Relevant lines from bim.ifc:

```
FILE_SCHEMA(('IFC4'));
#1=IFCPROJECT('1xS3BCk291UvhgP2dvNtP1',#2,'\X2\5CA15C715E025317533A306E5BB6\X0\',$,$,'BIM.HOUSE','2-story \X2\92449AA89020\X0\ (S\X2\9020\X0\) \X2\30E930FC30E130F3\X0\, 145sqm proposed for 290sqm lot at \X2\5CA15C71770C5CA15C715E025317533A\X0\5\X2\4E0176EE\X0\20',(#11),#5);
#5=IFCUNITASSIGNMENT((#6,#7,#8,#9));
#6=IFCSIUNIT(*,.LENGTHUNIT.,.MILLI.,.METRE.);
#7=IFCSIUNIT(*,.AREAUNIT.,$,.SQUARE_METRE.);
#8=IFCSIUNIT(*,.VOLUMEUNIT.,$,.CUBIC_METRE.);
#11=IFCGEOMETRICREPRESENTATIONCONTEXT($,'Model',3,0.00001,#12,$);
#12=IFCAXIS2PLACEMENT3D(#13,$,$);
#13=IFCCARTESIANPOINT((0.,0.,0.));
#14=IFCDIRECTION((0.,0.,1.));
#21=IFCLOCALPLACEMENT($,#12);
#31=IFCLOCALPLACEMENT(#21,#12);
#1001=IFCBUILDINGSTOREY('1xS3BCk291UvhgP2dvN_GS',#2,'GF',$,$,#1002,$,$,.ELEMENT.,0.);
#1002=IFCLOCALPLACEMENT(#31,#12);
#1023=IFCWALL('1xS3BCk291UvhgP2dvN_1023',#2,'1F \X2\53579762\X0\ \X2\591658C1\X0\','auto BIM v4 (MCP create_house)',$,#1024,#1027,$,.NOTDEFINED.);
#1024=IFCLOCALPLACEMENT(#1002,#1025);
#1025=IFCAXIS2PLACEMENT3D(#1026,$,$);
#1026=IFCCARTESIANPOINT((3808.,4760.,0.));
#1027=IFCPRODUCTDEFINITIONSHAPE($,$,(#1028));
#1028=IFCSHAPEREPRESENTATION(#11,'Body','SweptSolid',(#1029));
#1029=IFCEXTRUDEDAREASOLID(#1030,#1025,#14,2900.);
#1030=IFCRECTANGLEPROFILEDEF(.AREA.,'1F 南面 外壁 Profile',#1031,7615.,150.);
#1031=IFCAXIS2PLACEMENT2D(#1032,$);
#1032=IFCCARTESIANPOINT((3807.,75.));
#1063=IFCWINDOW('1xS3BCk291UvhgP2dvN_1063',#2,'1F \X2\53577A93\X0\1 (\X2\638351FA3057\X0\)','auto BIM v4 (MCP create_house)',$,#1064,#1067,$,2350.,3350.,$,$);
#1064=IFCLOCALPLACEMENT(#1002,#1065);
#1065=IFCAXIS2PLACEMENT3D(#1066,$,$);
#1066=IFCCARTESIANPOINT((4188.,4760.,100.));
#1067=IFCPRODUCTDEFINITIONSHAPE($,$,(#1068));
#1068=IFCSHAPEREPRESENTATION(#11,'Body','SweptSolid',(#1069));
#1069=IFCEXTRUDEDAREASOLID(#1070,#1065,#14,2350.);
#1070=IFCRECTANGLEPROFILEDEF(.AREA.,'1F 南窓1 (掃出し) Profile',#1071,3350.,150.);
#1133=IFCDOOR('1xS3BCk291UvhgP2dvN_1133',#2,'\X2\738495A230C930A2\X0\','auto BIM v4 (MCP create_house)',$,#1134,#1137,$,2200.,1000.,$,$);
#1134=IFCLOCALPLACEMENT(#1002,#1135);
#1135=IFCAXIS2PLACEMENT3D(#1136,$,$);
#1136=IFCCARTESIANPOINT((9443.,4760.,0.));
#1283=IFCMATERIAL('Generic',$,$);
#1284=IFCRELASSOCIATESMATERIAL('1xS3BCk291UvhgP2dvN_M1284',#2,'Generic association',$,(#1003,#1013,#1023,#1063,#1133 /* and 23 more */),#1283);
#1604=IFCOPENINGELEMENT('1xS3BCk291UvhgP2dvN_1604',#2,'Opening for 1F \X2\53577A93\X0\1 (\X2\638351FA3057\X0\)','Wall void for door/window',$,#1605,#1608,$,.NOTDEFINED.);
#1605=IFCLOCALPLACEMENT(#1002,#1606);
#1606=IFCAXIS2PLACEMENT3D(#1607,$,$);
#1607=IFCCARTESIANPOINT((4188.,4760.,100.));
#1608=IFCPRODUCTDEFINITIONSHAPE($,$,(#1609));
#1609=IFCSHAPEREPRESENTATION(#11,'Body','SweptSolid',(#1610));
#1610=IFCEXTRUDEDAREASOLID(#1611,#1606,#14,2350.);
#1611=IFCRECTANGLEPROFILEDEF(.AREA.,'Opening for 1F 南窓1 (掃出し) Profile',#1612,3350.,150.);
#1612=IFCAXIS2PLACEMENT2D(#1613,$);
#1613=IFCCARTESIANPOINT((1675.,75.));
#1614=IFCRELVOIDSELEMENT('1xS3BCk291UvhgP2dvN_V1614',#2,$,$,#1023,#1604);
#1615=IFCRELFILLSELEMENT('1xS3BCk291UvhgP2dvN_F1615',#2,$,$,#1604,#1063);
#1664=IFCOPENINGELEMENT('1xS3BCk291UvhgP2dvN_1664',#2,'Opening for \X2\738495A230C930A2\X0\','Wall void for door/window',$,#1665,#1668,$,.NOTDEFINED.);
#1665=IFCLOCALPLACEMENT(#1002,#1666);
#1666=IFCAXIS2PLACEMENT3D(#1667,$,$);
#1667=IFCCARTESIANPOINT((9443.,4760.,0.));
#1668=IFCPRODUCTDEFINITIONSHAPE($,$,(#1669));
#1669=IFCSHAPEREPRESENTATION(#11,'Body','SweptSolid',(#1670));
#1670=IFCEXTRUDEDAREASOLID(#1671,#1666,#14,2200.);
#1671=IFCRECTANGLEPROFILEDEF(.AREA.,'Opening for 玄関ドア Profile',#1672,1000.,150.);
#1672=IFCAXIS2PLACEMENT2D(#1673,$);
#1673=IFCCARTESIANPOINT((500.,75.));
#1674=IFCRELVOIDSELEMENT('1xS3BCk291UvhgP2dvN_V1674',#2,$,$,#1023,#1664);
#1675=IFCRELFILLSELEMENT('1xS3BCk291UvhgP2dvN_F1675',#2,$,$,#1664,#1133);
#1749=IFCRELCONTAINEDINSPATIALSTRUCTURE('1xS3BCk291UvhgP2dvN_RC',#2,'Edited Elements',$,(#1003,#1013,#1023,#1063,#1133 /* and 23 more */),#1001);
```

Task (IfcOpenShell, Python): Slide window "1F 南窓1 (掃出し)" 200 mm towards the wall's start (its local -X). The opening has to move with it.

```python
import ifcopenshell
import ifcopenshell.api.geometry
import ifcopenshell.util.placement

model = ifcopenshell.open("bim.ifc")

window = model.by_guid("1xS3BCk291UvhgP2dvN_1063")
opening = window.FillsVoids[0].RelatingOpeningElement
wall = opening.VoidsElements[0].RelatingBuildingElement

wall_matrix = ifcopenshell.util.placement.get_local_placement(wall.ObjectPlacement)
shift = wall_matrix[:3, 0] * -200.0
before = ifcopenshell.util.placement.get_local_placement(window.ObjectPlacement)[:3, 3].copy()

# The window is not placed relative to its opening, so move both.
for product in (opening, window):
    matrix = ifcopenshell.util.placement.get_local_placement(product.ObjectPlacement)
    matrix[:3, 3] += shift
    ifcopenshell.api.geometry.edit_object_placement(model, product=product, matrix=matrix, is_si=False)

after = ifcopenshell.util.placement.get_local_placement(window.ObjectPlacement)[:3, 3]
print("window moved by", (after - before).round(3) + 0.0)

model.write("bim_edited.ifc")
```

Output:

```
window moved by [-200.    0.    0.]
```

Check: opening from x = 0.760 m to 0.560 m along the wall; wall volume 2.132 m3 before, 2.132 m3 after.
